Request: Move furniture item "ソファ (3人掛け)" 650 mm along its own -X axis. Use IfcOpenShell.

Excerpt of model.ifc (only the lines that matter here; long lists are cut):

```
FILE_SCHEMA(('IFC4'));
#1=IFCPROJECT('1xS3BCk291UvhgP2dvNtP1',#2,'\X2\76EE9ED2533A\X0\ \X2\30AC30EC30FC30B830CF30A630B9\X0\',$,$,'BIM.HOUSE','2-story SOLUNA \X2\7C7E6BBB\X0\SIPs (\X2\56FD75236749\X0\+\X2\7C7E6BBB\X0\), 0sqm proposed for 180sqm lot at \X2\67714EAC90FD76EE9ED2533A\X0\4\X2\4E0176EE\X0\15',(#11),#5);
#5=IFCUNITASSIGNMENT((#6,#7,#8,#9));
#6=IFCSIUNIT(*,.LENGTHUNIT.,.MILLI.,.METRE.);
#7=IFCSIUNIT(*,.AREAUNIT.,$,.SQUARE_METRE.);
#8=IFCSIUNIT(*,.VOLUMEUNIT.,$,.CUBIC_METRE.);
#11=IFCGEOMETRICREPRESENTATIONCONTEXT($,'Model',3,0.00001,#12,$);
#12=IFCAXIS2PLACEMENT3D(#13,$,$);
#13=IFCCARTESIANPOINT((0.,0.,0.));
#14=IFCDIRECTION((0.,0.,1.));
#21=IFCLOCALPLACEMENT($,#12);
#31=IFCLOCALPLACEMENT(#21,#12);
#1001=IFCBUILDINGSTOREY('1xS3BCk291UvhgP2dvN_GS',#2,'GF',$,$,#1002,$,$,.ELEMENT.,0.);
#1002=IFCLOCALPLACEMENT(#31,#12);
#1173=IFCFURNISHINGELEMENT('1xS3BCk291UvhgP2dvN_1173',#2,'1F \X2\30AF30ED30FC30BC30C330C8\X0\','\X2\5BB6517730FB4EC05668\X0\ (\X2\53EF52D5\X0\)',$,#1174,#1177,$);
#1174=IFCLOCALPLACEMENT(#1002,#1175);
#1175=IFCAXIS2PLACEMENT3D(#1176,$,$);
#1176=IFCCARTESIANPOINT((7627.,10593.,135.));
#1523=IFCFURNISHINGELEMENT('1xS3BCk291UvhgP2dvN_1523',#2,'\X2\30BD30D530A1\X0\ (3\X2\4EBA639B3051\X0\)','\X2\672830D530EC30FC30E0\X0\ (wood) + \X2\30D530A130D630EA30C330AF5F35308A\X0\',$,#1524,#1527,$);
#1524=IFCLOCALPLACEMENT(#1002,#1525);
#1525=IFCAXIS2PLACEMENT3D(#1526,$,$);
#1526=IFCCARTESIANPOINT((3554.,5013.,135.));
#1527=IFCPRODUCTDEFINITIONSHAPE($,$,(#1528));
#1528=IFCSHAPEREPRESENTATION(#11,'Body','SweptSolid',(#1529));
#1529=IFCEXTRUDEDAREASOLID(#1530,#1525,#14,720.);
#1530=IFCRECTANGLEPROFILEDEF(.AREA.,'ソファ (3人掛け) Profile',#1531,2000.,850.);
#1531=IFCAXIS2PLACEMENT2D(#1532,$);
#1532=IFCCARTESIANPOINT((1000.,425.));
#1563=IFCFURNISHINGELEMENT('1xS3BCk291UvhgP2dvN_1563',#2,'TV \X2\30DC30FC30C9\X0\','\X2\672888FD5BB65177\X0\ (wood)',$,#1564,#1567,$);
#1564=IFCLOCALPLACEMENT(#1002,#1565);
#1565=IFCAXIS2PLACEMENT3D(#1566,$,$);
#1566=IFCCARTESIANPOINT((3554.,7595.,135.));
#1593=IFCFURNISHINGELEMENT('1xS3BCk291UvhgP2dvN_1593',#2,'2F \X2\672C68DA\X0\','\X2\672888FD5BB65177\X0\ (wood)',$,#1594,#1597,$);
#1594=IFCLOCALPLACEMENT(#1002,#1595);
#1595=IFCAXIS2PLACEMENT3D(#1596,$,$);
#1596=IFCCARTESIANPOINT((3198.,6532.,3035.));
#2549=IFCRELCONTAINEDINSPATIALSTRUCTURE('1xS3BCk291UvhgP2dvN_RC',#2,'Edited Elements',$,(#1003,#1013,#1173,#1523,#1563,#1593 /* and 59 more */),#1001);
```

```python
import ifcopenshell
import ifcopenshell.api.geometry
import ifcopenshell.util.placement

model = ifcopenshell.open("model.ifc")

item = model.by_guid("1xS3BCk291UvhgP2dvN_1523")
matrix = ifcopenshell.util.placement.get_local_placement(item.ObjectPlacement)
matrix[:3, 3] -= matrix[:3, 0] * 650.0
ifcopenshell.api.geometry.edit_object_placement(model, product=item, matrix=matrix, is_si=False)

print(ifcopenshell.util.placement.get_local_placement(item.ObjectPlacement).round(3) + 0.0)

model.write("model_edited.ifc")
```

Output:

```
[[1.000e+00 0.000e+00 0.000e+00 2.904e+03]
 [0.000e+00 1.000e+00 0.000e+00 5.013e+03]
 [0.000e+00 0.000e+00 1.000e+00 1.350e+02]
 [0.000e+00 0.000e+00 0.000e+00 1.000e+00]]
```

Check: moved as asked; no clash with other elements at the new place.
